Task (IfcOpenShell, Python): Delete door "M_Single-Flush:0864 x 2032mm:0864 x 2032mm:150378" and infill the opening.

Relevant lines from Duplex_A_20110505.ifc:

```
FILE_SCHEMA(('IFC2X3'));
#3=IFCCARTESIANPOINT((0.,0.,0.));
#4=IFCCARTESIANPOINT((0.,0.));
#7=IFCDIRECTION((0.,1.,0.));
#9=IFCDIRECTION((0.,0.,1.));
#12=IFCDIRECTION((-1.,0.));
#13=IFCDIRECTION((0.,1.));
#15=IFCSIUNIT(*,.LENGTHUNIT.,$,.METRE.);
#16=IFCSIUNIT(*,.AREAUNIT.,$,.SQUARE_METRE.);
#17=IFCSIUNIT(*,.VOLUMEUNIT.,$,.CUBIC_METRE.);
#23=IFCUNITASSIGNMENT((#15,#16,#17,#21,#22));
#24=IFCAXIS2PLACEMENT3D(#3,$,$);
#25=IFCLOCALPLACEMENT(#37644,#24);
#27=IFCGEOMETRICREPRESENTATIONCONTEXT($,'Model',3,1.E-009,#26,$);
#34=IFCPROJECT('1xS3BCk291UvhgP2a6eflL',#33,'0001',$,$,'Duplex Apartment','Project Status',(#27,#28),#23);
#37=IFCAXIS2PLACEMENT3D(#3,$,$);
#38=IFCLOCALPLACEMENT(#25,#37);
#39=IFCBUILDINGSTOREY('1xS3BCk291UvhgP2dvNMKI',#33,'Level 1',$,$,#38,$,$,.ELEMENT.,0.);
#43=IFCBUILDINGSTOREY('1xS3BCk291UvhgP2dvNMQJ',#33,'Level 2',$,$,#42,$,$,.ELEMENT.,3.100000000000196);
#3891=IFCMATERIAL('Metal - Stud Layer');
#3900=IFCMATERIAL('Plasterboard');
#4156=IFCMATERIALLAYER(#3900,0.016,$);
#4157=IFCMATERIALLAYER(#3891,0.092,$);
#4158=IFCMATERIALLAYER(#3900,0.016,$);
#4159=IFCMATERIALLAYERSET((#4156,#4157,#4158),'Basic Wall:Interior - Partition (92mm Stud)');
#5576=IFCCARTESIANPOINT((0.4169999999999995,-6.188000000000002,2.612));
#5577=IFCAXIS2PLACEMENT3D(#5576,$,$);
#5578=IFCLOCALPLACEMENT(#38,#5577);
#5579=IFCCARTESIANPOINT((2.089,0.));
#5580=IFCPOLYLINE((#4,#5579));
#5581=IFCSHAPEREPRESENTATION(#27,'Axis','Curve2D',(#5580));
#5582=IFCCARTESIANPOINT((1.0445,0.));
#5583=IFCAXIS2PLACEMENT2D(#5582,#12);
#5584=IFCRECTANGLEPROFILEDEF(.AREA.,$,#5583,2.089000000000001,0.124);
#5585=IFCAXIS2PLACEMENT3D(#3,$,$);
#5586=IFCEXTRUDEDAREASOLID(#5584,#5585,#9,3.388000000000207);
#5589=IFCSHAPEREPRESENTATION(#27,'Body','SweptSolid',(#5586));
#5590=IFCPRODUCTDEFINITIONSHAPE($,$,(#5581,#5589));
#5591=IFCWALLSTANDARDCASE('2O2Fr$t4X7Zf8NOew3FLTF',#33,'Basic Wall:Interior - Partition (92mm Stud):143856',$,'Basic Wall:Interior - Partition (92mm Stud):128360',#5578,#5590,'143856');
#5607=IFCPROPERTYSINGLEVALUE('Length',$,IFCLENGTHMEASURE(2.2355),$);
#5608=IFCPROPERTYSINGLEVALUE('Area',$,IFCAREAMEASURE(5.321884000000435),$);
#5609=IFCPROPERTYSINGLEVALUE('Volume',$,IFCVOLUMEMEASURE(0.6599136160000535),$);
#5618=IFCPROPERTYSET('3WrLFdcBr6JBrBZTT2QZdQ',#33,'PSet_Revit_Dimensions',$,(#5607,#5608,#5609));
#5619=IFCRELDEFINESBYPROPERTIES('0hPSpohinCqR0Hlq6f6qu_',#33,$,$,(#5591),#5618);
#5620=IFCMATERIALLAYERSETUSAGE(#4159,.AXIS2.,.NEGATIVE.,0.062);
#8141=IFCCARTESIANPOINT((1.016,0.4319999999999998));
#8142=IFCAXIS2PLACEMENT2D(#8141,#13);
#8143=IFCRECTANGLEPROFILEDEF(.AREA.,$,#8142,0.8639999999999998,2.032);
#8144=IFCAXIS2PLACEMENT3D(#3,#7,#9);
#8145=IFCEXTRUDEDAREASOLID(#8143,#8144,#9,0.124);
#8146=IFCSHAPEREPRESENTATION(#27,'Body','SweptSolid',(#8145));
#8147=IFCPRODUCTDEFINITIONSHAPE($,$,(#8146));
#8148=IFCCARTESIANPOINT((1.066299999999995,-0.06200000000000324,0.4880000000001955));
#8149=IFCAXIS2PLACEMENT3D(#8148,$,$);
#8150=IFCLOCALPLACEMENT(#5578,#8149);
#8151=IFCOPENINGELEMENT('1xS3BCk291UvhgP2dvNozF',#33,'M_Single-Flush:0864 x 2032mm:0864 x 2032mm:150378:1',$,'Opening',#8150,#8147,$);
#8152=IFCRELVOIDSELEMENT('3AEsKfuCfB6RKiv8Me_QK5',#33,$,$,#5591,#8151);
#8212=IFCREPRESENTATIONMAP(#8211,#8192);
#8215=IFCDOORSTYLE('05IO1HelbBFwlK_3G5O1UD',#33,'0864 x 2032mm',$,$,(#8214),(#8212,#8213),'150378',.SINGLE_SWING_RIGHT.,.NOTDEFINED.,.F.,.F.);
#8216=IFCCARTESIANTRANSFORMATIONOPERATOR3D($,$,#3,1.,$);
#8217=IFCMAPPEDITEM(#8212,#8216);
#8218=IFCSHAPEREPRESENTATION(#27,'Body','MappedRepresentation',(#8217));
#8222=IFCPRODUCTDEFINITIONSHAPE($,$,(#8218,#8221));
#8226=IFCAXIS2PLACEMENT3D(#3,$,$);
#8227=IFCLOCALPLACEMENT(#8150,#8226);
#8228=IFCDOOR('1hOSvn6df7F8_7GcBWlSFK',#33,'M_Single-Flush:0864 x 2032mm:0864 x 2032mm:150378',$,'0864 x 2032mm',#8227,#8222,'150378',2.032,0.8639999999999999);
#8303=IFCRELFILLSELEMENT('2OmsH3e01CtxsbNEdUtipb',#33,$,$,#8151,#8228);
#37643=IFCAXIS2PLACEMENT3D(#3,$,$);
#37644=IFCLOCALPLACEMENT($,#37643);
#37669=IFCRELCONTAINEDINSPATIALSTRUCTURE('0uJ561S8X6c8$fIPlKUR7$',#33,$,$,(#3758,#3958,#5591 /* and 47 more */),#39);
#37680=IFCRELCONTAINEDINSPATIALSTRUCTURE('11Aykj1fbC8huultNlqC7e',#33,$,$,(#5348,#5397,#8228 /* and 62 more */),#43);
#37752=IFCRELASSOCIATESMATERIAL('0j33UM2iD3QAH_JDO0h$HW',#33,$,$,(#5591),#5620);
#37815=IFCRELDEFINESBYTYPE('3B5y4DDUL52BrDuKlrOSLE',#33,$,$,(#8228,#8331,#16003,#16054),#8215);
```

```python
import ifcopenshell
import ifcopenshell.api.feature
import ifcopenshell.api.pset
import ifcopenshell.api.root
import ifcopenshell.geom
import ifcopenshell.util.element
import ifcopenshell.util.shape
import ifcopenshell.util.unit

model = ifcopenshell.open("Duplex_A_20110505.ifc")
area_scale = ifcopenshell.util.unit.calculate_unit_scale(model, "AREAUNIT")
volume_scale = ifcopenshell.util.unit.calculate_unit_scale(model, "VOLUMEUNIT")
settings = ifcopenshell.geom.settings()


def volume(element):
    """Net volume in cubic metres, openings subtracted."""
    shape = ifcopenshell.geom.create_shape(settings, element)
    return ifcopenshell.util.shape.get_volume(shape.geometry)


door = model.by_id(8228)
opening = door.FillsVoids[0].RelatingOpeningElement
wall = opening.VoidsElements[0].RelatingBuildingElement
before = volume(wall)

ifcopenshell.api.root.remove_product(model, product=door)
ifcopenshell.api.feature.remove_feature(model, feature=opening)

after = volume(wall)
thickness = 0.124  # wall thickness in metres

# Update the wall's stored quantities.
pset = model.by_id(ifcopenshell.util.element.get_pset(wall, "PSet_Revit_Dimensions", should_inherit=False)["id"])
ifcopenshell.api.pset.edit_pset(model, pset=pset, properties={
    "Area": model.create_entity("IfcAreaMeasure", after / thickness / area_scale),
    "Volume": model.create_entity("IfcVolumeMeasure", after / volume_scale),
})

print(f"wall volume {before:.3f} -> {after:.3f} m3")

model.write("Duplex_A_20110505_edited.ifc")
```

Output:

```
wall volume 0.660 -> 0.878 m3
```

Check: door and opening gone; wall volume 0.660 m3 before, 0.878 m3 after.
